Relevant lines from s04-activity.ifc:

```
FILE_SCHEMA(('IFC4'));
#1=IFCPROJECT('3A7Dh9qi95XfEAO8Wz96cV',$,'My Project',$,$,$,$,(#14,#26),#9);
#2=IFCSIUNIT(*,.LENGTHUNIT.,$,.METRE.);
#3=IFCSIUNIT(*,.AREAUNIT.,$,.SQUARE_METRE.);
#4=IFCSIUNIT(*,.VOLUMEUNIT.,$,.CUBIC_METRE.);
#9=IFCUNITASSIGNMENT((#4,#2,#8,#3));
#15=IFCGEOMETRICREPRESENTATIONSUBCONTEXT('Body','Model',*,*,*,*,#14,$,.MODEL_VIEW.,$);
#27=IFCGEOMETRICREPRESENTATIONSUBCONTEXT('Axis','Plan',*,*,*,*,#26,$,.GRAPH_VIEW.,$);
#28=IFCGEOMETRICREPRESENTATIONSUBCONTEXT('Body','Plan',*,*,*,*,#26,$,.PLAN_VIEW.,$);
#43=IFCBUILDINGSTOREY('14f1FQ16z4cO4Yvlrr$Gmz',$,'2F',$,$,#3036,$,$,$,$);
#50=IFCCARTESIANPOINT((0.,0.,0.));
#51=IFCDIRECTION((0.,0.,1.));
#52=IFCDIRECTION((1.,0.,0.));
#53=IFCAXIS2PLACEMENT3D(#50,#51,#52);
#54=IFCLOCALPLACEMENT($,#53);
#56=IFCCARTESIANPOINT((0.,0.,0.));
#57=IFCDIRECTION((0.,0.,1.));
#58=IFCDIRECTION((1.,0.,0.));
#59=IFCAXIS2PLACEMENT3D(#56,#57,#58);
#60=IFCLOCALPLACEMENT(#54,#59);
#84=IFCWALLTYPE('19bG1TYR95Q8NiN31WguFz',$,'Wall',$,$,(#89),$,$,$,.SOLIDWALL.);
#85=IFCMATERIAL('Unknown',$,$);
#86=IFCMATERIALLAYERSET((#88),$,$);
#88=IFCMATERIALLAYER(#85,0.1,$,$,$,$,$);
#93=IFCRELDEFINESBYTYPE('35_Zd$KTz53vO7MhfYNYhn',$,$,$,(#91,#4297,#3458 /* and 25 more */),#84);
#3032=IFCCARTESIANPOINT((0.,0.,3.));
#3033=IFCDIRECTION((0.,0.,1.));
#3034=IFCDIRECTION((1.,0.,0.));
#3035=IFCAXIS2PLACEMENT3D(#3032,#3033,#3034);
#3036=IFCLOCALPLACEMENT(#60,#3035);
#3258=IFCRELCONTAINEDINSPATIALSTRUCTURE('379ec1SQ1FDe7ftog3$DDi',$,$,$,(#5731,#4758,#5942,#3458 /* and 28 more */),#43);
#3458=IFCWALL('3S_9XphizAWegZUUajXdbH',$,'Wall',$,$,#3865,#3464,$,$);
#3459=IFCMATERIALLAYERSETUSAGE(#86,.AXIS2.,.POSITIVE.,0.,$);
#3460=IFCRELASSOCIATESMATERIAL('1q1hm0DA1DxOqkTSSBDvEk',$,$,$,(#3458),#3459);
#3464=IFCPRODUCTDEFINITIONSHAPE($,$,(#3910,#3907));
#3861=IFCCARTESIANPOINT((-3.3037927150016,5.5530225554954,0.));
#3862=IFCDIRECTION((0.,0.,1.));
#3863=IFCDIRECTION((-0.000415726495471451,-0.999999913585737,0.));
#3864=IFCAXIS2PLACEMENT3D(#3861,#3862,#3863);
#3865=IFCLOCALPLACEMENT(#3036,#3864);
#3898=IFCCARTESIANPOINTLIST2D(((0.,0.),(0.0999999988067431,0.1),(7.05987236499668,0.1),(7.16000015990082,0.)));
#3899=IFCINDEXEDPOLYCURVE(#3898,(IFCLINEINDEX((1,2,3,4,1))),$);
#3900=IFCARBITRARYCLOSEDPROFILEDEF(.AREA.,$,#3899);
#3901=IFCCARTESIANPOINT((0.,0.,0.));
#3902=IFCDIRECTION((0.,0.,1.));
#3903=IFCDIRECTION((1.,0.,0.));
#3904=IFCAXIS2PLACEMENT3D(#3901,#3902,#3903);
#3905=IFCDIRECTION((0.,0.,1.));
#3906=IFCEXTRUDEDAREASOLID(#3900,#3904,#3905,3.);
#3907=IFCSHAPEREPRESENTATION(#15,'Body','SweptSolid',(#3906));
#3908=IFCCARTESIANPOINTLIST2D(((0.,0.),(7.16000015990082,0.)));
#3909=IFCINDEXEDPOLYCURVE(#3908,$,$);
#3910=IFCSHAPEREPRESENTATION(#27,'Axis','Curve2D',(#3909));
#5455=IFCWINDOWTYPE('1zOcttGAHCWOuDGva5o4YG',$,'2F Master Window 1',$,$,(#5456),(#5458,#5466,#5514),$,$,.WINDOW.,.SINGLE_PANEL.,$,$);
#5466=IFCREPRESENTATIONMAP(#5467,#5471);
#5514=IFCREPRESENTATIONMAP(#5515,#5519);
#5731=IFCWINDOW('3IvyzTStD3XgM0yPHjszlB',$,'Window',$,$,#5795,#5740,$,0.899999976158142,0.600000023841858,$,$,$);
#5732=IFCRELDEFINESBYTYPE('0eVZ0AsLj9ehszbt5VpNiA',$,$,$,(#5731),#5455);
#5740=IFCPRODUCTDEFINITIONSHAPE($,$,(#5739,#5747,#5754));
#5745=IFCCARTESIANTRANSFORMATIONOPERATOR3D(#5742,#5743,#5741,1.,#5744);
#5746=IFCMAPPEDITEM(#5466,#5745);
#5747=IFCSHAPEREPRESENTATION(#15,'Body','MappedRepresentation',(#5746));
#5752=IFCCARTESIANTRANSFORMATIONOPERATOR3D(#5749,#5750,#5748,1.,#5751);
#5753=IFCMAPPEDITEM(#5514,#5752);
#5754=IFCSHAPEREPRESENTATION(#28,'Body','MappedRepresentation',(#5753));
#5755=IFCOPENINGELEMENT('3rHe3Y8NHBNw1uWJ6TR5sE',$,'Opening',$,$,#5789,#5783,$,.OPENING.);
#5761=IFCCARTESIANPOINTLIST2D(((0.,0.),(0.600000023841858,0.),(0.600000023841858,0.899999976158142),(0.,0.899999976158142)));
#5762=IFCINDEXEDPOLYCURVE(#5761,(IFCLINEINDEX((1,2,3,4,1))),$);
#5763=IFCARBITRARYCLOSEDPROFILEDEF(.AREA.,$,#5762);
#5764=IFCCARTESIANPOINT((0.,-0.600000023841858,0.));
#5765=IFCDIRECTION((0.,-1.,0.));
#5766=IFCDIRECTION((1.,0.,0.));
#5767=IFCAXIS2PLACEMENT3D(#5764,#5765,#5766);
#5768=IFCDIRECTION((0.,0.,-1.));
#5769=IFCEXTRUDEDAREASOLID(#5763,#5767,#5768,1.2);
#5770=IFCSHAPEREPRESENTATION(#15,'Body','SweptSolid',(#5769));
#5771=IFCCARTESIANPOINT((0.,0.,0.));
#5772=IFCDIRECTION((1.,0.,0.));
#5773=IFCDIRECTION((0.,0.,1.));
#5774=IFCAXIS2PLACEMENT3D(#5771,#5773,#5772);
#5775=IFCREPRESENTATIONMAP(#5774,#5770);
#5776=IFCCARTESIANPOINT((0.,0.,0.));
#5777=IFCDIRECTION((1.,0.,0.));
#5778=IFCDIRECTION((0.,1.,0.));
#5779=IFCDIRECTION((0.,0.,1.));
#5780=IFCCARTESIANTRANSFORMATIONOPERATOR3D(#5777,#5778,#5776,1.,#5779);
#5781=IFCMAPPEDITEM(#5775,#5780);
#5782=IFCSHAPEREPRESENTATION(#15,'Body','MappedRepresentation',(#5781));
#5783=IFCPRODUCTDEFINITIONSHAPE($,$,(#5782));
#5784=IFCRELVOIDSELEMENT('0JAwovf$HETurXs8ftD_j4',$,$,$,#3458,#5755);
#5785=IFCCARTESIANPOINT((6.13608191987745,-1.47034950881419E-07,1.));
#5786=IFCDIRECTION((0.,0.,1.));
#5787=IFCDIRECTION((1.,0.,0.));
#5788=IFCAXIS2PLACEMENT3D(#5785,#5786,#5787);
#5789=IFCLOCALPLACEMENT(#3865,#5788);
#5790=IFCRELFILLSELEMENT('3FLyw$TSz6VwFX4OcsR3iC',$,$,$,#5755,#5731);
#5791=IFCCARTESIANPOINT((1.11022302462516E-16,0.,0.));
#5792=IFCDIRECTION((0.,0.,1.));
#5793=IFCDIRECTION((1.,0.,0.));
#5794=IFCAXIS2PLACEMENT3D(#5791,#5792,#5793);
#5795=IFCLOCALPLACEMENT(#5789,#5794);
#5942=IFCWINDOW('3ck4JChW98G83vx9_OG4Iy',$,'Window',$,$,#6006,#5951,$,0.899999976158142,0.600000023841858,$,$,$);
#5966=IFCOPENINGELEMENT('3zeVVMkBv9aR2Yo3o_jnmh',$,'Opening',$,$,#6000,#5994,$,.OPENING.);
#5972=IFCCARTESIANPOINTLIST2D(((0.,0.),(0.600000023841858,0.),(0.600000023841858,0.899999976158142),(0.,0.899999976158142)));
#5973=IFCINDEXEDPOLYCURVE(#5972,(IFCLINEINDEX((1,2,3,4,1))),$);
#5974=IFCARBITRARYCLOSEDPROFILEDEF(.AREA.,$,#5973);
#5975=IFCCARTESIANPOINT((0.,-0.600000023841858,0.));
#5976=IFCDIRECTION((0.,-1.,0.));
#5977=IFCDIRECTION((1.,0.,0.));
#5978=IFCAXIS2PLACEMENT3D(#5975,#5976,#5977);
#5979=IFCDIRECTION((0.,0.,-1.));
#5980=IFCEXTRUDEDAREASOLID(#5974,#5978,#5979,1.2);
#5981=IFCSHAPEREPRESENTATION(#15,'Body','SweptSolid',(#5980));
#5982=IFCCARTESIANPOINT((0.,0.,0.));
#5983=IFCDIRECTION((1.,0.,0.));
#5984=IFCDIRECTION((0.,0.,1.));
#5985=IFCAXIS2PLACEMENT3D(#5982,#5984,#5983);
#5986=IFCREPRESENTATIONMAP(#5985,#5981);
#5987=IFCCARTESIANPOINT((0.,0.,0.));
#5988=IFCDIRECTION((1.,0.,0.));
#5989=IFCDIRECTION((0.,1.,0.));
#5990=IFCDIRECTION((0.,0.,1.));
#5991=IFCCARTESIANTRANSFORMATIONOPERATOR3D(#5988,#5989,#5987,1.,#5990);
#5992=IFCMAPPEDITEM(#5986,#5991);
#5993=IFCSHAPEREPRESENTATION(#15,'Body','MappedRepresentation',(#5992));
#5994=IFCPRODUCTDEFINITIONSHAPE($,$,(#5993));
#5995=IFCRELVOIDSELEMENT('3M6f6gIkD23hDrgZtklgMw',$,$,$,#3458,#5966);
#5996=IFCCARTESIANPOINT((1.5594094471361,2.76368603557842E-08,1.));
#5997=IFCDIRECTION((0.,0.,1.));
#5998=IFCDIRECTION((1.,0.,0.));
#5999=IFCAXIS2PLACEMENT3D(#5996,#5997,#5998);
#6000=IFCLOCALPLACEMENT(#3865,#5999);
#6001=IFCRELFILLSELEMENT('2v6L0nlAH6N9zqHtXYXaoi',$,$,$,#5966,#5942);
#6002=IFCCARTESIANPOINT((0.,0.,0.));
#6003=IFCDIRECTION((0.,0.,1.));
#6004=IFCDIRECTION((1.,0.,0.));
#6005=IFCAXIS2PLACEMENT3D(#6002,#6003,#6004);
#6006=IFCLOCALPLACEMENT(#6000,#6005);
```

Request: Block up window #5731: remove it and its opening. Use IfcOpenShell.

```python
import ifcopenshell
import ifcopenshell.api.feature
import ifcopenshell.api.root
import ifcopenshell.geom
import ifcopenshell.util.shape

model = ifcopenshell.open("s04-activity.ifc")
settings = ifcopenshell.geom.settings()


def volume(element):
    """Net volume in cubic metres, openings subtracted."""
    shape = ifcopenshell.geom.create_shape(settings, element)
    return ifcopenshell.util.shape.get_volume(shape.geometry)


window = model.by_guid("3IvyzTStD3XgM0yPHjszlB")
opening = window.FillsVoids[0].RelatingOpeningElement
wall = opening.VoidsElements[0].RelatingBuildingElement
before = volume(wall)

ifcopenshell.api.root.remove_product(model, product=window)
ifcopenshell.api.feature.remove_feature(model, feature=opening)

after = volume(wall)

print(f"wall volume {before:.3f} -> {after:.3f} m3")

model.write("s04-activity_updated.ifc")
```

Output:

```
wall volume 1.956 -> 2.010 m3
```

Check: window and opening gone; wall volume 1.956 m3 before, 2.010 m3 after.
